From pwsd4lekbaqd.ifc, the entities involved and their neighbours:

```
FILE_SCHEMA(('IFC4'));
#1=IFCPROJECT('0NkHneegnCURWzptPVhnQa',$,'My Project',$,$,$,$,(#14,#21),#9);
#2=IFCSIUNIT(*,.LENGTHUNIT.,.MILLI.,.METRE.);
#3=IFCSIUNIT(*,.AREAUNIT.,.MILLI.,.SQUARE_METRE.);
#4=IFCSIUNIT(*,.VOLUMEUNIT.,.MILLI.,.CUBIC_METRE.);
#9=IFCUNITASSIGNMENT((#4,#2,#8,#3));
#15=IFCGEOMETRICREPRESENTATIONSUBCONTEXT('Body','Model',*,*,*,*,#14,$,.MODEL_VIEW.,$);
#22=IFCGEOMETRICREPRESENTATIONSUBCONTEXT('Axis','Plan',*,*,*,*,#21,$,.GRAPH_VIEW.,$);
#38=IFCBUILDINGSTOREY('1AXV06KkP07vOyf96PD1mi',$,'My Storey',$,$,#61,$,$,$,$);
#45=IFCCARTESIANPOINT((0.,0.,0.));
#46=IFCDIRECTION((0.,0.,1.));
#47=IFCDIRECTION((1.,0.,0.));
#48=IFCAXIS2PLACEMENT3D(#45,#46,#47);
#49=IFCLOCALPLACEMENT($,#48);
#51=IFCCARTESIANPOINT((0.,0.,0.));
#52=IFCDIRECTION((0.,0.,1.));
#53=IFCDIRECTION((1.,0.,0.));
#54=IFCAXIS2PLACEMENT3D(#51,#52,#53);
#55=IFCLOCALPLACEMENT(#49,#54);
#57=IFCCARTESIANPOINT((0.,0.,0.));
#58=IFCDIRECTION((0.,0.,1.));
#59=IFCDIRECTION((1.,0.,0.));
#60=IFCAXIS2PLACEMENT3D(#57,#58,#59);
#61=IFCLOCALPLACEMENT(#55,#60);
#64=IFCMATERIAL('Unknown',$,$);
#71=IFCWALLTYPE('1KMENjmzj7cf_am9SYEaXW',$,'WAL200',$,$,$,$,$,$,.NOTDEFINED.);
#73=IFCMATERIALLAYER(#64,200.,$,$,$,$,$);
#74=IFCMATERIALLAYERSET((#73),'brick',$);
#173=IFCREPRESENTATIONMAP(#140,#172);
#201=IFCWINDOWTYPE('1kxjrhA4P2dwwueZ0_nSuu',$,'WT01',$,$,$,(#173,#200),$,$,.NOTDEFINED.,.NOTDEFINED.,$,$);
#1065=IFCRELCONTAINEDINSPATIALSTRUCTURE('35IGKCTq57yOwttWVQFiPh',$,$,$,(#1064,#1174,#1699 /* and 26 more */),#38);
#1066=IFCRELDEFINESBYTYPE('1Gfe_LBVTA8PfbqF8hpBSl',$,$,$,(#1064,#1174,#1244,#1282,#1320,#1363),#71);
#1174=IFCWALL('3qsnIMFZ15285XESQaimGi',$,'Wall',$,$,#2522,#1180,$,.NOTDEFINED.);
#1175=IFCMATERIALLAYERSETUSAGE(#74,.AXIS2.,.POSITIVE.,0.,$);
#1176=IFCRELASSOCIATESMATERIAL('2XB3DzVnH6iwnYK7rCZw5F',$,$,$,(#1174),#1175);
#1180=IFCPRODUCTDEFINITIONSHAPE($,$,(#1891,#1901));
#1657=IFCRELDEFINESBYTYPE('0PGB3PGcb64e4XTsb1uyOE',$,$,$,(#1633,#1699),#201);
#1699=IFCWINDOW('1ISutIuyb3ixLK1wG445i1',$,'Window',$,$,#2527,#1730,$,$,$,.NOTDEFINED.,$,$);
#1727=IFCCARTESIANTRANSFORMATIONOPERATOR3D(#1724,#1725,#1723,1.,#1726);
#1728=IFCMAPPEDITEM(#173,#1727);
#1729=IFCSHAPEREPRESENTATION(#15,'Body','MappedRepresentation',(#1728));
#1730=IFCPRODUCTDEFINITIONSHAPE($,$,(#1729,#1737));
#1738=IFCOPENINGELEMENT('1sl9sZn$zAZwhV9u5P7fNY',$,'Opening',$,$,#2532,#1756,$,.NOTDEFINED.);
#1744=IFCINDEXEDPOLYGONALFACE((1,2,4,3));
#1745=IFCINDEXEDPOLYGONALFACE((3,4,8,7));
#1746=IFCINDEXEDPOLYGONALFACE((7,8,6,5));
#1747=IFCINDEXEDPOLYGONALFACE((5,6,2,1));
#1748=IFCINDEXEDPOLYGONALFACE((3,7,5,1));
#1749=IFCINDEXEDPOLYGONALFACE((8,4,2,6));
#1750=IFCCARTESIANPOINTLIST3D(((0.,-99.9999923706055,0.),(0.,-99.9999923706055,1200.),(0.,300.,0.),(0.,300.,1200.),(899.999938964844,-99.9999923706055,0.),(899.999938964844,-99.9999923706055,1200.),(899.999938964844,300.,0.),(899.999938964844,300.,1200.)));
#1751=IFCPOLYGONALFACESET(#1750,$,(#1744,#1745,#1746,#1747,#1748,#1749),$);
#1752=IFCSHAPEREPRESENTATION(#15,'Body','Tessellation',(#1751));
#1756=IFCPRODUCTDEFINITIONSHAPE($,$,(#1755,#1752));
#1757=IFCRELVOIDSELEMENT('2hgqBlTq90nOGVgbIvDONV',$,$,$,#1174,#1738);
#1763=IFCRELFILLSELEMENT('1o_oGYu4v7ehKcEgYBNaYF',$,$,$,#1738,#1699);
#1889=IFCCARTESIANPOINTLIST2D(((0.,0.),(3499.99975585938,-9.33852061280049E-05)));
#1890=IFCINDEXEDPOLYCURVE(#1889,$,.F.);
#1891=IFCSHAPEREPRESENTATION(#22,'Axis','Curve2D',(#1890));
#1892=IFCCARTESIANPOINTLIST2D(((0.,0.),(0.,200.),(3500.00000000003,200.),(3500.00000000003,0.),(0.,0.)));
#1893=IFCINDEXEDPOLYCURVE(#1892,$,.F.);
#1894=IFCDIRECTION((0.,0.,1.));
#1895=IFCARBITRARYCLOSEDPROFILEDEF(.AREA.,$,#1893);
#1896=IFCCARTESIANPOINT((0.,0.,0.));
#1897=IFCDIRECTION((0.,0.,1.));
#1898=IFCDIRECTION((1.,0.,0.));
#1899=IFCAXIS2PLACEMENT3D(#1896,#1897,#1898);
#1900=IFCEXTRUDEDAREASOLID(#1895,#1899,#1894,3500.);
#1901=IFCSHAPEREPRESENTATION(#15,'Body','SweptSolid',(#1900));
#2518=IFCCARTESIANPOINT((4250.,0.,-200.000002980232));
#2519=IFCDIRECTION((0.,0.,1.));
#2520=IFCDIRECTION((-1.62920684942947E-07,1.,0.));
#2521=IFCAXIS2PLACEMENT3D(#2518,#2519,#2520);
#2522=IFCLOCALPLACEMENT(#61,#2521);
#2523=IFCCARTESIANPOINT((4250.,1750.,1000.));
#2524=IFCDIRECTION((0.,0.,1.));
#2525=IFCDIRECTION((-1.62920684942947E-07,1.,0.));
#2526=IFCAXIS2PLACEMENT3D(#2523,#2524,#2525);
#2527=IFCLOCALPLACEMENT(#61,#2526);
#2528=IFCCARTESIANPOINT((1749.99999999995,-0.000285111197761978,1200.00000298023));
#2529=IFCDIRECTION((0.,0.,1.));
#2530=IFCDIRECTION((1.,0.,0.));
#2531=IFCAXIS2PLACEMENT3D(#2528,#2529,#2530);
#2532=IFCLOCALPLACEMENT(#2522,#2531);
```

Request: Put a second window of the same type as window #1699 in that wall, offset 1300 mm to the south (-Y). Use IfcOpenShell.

```python
import ifcopenshell
import ifcopenshell.api.feature
import ifcopenshell.api.geometry
import ifcopenshell.api.root
import ifcopenshell.geom
import ifcopenshell.util.element
import ifcopenshell.util.placement
import ifcopenshell.util.shape

model = ifcopenshell.open("pwsd4lekbaqd.ifc")
settings = ifcopenshell.geom.settings()


def volume(element):
    """Net volume in cubic metres, openings subtracted."""
    shape = ifcopenshell.geom.create_shape(settings, element)
    return ifcopenshell.util.shape.get_volume(shape.geometry)


window = model.by_guid("1ISutIuyb3ixLK1wG445i1")
opening = window.FillsVoids[0].RelatingOpeningElement
wall = opening.VoidsElements[0].RelatingBuildingElement
before = volume(wall)
shift = ifcopenshell.util.placement.get_local_placement(wall.ObjectPlacement)[:3, 0] * -1300.0

# copy_class copies the void relationship, type, container and properties, but no geometry.
new_opening = ifcopenshell.api.root.copy_class(model, product=opening)
new_opening.Representation = ifcopenshell.util.element.copy_deep(
    model, opening.Representation, exclude=["IfcGeometricRepresentationContext", "IfcRepresentationMap"]
)
new_window = ifcopenshell.api.root.copy_class(model, product=window)
new_window.Representation = ifcopenshell.util.element.copy_deep(
    model, window.Representation, exclude=["IfcGeometricRepresentationContext", "IfcRepresentationMap"]
)
ifcopenshell.api.feature.add_filling(model, opening=new_opening, element=new_window)

for old, new in ((opening, new_opening), (window, new_window)):
    matrix = ifcopenshell.util.placement.get_local_placement(old.ObjectPlacement)
    matrix[:3, 3] += shift
    ifcopenshell.api.geometry.edit_object_placement(model, product=new, matrix=matrix, is_si=False)

after = volume(wall)

print(f"wall volume {before:.3f} -> {after:.3f} m3")

model.write("pwsd4lekbaqd_updated.ifc")
```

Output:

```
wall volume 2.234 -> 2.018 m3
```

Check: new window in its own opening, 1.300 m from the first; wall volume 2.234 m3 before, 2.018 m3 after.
